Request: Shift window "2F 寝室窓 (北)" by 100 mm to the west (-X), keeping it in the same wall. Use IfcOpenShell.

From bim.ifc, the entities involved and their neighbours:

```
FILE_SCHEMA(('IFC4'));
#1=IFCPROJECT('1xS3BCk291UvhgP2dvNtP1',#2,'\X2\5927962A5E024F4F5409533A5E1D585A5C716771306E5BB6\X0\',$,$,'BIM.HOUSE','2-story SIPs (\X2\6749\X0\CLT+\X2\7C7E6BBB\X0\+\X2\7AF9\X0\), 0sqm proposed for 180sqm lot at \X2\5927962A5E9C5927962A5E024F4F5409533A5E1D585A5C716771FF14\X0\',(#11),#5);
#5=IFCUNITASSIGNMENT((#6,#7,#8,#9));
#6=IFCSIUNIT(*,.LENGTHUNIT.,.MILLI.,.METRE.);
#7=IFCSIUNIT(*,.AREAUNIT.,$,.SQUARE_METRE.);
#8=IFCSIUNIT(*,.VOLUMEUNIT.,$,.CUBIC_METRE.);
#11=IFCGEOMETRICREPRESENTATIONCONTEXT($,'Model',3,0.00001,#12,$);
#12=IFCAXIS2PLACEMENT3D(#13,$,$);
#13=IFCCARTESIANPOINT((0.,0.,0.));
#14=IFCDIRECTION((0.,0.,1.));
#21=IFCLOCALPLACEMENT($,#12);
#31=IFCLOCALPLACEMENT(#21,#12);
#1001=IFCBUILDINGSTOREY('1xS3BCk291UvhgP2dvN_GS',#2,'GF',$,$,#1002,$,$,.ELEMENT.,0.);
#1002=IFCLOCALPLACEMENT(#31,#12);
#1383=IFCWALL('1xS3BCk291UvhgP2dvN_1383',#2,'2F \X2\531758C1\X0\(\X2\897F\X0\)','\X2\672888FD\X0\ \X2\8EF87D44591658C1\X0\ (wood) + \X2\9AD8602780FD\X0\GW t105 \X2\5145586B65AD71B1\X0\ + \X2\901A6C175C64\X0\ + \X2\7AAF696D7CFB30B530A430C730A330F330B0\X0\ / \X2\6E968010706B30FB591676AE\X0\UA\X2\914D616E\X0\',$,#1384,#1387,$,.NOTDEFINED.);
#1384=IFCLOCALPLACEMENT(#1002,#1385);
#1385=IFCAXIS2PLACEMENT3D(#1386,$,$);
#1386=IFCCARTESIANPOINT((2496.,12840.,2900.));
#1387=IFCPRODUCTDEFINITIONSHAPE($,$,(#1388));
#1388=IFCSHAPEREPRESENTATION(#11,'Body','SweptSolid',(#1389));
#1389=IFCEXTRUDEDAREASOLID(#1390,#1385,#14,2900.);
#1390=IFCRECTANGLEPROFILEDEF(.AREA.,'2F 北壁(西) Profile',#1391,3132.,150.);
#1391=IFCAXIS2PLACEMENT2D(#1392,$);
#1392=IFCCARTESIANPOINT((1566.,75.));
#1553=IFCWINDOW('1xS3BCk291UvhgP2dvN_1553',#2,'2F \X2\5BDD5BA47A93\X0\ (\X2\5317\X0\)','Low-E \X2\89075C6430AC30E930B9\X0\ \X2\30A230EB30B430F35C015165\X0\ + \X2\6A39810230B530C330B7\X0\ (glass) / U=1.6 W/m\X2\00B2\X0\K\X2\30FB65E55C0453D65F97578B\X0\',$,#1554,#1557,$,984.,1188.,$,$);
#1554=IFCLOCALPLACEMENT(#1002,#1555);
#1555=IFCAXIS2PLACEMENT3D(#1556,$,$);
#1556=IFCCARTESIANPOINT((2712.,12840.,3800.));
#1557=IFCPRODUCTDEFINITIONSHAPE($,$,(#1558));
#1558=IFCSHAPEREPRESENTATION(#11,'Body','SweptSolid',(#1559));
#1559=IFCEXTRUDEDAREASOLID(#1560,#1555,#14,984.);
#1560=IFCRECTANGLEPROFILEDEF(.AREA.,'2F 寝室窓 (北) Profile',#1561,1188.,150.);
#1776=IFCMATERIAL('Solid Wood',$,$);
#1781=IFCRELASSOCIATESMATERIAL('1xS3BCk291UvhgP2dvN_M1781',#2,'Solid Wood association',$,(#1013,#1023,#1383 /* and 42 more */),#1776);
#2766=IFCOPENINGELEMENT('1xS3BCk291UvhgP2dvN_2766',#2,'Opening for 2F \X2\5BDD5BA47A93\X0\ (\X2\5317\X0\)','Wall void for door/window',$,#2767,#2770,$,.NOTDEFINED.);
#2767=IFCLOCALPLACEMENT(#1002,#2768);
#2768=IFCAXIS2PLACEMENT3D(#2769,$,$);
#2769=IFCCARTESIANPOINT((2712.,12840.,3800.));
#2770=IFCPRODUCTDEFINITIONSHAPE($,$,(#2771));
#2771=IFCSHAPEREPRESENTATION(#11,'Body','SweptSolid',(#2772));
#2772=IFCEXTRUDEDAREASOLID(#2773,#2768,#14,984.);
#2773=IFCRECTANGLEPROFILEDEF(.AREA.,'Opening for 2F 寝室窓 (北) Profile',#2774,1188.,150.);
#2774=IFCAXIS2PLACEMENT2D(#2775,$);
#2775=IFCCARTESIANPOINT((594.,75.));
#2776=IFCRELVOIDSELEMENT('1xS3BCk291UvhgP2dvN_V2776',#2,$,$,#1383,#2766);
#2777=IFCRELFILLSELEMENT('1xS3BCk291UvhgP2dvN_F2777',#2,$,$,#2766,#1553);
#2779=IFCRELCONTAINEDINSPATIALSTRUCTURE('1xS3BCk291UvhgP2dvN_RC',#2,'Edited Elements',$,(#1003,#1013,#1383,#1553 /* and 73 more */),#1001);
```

```python
import ifcopenshell
import ifcopenshell.api.geometry
import ifcopenshell.util.placement
import ifcopenshell.util.unit

model = ifcopenshell.open("bim.ifc")
unit_scale = ifcopenshell.util.unit.calculate_unit_scale(model)

window = model.by_guid("1xS3BCk291UvhgP2dvN_1553")
opening = window.FillsVoids[0].RelatingOpeningElement
wall = opening.VoidsElements[0].RelatingBuildingElement

wall_matrix = ifcopenshell.util.placement.get_local_placement(wall.ObjectPlacement)
shift = wall_matrix[:3, 0] * -0.1 / unit_scale
before = ifcopenshell.util.placement.get_local_placement(window.ObjectPlacement)[:3, 3].copy()

# The window is not placed relative to its opening, so move both.
for product in (opening, window):
    matrix = ifcopenshell.util.placement.get_local_placement(product.ObjectPlacement)
    matrix[:3, 3] += shift
    ifcopenshell.api.geometry.edit_object_placement(model, product=product, matrix=matrix, is_si=False)

after = ifcopenshell.util.placement.get_local_placement(window.ObjectPlacement)[:3, 3]
print("window moved by", (after - before).round(3) + 0.0)

model.write("bim-out.ifc")
```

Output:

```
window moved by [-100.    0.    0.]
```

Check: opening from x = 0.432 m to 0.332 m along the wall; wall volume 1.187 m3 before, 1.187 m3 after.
